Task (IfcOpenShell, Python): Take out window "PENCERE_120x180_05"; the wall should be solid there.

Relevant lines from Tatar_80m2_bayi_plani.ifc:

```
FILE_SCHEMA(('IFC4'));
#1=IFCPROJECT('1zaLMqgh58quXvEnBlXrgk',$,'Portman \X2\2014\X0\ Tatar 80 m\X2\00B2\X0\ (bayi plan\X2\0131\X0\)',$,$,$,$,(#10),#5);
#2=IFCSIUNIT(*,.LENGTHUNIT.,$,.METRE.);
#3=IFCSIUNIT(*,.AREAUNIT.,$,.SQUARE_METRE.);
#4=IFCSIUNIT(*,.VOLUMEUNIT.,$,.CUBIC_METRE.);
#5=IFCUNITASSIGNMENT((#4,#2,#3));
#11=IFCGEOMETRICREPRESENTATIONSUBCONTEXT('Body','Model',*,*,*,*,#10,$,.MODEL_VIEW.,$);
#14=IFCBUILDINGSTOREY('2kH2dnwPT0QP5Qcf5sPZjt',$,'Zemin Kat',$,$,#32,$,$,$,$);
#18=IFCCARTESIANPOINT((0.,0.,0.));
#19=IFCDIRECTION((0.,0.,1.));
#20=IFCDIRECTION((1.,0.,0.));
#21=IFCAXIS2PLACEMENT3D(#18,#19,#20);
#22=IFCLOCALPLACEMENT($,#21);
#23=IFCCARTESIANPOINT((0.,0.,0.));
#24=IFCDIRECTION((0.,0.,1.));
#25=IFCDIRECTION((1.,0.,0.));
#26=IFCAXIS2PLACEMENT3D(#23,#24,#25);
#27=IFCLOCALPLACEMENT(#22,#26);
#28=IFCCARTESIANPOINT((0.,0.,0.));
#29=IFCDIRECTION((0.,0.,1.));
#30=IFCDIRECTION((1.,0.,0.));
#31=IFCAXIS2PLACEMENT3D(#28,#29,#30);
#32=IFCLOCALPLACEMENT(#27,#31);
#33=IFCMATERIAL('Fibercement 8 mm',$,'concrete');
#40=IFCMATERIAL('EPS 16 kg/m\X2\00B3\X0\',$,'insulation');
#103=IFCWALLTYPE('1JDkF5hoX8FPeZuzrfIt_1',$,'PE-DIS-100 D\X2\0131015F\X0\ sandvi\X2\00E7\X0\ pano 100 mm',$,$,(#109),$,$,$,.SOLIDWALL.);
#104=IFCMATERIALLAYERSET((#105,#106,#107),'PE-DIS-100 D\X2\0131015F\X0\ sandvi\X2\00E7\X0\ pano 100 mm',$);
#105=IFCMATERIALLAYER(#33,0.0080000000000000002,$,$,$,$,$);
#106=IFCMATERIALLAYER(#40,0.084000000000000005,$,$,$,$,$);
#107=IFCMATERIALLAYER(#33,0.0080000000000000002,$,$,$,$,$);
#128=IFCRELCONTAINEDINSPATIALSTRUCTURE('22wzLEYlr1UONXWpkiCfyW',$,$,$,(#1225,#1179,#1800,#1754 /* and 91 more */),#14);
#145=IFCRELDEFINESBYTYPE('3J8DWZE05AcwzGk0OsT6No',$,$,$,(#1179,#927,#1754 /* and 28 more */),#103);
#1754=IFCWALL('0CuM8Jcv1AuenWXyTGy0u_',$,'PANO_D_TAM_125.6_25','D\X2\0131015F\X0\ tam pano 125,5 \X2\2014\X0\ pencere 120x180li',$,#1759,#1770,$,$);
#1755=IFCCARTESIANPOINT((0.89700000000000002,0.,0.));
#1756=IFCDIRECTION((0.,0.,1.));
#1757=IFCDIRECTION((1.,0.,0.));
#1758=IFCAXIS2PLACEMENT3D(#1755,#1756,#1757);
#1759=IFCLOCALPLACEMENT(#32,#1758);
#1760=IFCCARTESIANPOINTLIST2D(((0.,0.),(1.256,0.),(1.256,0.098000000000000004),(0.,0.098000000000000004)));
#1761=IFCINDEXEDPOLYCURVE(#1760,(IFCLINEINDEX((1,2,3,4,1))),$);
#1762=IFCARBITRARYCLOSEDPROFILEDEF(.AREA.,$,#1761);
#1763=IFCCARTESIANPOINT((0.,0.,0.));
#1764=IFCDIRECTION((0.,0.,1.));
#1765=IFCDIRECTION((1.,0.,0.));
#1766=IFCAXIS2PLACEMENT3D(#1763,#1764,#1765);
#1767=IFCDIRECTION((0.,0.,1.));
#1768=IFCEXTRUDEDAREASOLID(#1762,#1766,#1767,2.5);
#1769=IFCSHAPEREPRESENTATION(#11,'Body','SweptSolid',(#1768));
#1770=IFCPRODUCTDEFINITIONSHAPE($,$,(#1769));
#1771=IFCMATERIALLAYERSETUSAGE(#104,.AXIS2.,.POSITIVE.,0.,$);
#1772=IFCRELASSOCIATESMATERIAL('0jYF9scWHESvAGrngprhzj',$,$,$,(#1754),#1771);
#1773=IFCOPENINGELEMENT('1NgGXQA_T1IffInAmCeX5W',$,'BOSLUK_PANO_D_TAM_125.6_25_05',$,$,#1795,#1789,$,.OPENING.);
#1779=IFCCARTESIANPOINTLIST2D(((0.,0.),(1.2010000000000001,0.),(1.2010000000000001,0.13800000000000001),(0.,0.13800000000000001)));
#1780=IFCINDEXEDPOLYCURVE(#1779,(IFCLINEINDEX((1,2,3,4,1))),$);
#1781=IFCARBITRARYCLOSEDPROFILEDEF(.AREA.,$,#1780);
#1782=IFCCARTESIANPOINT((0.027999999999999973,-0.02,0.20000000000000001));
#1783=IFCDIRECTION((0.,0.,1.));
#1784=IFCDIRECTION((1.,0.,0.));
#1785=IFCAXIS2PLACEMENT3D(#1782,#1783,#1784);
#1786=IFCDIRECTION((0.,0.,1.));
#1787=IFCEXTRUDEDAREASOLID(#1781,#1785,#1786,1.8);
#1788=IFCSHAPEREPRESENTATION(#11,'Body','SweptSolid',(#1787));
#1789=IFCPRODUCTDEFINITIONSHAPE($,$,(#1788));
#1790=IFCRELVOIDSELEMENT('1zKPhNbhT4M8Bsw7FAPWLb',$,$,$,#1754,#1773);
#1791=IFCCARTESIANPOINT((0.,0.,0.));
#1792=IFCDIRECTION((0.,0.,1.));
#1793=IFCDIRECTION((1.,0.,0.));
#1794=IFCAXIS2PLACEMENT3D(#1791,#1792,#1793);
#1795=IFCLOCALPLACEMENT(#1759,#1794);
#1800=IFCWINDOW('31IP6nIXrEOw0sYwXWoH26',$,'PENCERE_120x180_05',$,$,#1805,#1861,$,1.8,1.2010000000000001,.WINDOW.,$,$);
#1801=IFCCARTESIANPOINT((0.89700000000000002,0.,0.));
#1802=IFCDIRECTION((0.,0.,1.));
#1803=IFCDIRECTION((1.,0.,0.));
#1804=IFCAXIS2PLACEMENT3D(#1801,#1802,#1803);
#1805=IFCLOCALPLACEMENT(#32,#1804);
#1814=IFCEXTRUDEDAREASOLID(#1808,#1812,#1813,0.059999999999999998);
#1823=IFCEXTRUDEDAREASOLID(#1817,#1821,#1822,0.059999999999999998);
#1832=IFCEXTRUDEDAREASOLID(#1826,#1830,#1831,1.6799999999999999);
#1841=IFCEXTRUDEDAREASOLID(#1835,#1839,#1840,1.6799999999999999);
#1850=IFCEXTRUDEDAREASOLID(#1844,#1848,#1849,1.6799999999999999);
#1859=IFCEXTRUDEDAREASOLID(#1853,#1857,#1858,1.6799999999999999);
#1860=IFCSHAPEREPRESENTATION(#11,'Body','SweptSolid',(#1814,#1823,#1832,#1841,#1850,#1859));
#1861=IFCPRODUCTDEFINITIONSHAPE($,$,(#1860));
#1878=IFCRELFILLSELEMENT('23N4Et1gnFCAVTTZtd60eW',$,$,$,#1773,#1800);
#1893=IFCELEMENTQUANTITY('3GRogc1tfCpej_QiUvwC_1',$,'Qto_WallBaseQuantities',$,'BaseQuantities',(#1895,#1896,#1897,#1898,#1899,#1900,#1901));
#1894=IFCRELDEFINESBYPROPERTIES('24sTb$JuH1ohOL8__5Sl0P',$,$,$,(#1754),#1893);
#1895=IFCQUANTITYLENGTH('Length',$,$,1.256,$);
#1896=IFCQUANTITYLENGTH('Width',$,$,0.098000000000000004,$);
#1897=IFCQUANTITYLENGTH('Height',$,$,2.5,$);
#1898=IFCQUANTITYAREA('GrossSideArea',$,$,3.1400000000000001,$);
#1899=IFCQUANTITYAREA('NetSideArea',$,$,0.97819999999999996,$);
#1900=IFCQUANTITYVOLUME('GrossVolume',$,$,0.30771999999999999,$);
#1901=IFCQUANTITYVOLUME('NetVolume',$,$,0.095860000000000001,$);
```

```python
import ifcopenshell
import ifcopenshell.api.feature
import ifcopenshell.api.pset
import ifcopenshell.api.root
import ifcopenshell.geom
import ifcopenshell.util.element
import ifcopenshell.util.shape
import ifcopenshell.util.unit

model = ifcopenshell.open("Tatar_80m2_bayi_plani.ifc")
area_scale = ifcopenshell.util.unit.calculate_unit_scale(model, "AREAUNIT")
volume_scale = ifcopenshell.util.unit.calculate_unit_scale(model, "VOLUMEUNIT")
settings = ifcopenshell.geom.settings()


def volume(element):
    """Net volume in cubic metres, openings subtracted."""
    shape = ifcopenshell.geom.create_shape(settings, element)
    return ifcopenshell.util.shape.get_volume(shape.geometry)


window = model.by_id(1800)
opening = window.FillsVoids[0].RelatingOpeningElement
wall = opening.VoidsElements[0].RelatingBuildingElement
before = volume(wall)

ifcopenshell.api.root.remove_product(model, product=window)
ifcopenshell.api.feature.remove_feature(model, feature=opening)

after = volume(wall)
thickness = 0.098  # wall thickness in metres

# Update the wall's stored quantities.
qto = model.by_id(ifcopenshell.util.element.get_pset(wall, "Qto_WallBaseQuantities", should_inherit=False)["id"])
ifcopenshell.api.pset.edit_qto(model, qto=qto, properties={
    "NetSideArea": after / thickness / area_scale,
    "NetVolume": after / volume_scale,
})

print(f"wall volume {before:.3f} -> {after:.3f} m3")

model.write("Tatar_80m2_bayi_plani_v2.ifc")
```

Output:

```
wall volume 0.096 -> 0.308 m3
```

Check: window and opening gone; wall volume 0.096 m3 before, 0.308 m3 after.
